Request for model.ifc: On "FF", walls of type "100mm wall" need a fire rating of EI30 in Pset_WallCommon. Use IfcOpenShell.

First a look at what the model holds.

```python
import ifcopenshell
import ifcopenshell.util.element

model = ifcopenshell.open("model.ifc")
print(model.schema)
storey = next(s for s in model.by_type("IfcBuildingStorey") if s.Name == "FF")
walls = [e for e in ifcopenshell.util.element.get_decomposition(storey) if e.is_a("IfcWall")]
seen = {}
for e in walls:
    element_type = ifcopenshell.util.element.get_type(e)
    key = (element_type.Name if element_type != e and element_type else None, ifcopenshell.util.element.get_pset(e, "Pset_WallCommon", "FireRating"))
    seen[key] = seen.get(key, 0) + 1
for (name, value), count in sorted(seen.items(), key=str):
    print(count, "x", name, "|", value)
```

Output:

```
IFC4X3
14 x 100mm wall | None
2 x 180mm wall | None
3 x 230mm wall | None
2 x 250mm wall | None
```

```python
import ifcopenshell
import ifcopenshell.api.pset
import ifcopenshell.util.element

model = ifcopenshell.open("model.ifc")

storey = next(s for s in model.by_type("IfcBuildingStorey") if s.Name == "FF")
walls = [e for e in ifcopenshell.util.element.get_decomposition(storey) if e.is_a("IfcWall")]

count = 0
for e in walls:
    element_type = ifcopenshell.util.element.get_type(e)
    if element_type in (None, e) or element_type.Name != "100mm wall":
        continue
    # add_pset returns the element's existing set when there is one.
    pset = ifcopenshell.api.pset.add_pset(model, product=e, name="Pset_WallCommon")
    ifcopenshell.api.pset.edit_pset(model, pset=pset, properties={"FireRating": "EI30"})
    count += 1

print(count, "walls updated")

model.write("model_edited.ifc")
```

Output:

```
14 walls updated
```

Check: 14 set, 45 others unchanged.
